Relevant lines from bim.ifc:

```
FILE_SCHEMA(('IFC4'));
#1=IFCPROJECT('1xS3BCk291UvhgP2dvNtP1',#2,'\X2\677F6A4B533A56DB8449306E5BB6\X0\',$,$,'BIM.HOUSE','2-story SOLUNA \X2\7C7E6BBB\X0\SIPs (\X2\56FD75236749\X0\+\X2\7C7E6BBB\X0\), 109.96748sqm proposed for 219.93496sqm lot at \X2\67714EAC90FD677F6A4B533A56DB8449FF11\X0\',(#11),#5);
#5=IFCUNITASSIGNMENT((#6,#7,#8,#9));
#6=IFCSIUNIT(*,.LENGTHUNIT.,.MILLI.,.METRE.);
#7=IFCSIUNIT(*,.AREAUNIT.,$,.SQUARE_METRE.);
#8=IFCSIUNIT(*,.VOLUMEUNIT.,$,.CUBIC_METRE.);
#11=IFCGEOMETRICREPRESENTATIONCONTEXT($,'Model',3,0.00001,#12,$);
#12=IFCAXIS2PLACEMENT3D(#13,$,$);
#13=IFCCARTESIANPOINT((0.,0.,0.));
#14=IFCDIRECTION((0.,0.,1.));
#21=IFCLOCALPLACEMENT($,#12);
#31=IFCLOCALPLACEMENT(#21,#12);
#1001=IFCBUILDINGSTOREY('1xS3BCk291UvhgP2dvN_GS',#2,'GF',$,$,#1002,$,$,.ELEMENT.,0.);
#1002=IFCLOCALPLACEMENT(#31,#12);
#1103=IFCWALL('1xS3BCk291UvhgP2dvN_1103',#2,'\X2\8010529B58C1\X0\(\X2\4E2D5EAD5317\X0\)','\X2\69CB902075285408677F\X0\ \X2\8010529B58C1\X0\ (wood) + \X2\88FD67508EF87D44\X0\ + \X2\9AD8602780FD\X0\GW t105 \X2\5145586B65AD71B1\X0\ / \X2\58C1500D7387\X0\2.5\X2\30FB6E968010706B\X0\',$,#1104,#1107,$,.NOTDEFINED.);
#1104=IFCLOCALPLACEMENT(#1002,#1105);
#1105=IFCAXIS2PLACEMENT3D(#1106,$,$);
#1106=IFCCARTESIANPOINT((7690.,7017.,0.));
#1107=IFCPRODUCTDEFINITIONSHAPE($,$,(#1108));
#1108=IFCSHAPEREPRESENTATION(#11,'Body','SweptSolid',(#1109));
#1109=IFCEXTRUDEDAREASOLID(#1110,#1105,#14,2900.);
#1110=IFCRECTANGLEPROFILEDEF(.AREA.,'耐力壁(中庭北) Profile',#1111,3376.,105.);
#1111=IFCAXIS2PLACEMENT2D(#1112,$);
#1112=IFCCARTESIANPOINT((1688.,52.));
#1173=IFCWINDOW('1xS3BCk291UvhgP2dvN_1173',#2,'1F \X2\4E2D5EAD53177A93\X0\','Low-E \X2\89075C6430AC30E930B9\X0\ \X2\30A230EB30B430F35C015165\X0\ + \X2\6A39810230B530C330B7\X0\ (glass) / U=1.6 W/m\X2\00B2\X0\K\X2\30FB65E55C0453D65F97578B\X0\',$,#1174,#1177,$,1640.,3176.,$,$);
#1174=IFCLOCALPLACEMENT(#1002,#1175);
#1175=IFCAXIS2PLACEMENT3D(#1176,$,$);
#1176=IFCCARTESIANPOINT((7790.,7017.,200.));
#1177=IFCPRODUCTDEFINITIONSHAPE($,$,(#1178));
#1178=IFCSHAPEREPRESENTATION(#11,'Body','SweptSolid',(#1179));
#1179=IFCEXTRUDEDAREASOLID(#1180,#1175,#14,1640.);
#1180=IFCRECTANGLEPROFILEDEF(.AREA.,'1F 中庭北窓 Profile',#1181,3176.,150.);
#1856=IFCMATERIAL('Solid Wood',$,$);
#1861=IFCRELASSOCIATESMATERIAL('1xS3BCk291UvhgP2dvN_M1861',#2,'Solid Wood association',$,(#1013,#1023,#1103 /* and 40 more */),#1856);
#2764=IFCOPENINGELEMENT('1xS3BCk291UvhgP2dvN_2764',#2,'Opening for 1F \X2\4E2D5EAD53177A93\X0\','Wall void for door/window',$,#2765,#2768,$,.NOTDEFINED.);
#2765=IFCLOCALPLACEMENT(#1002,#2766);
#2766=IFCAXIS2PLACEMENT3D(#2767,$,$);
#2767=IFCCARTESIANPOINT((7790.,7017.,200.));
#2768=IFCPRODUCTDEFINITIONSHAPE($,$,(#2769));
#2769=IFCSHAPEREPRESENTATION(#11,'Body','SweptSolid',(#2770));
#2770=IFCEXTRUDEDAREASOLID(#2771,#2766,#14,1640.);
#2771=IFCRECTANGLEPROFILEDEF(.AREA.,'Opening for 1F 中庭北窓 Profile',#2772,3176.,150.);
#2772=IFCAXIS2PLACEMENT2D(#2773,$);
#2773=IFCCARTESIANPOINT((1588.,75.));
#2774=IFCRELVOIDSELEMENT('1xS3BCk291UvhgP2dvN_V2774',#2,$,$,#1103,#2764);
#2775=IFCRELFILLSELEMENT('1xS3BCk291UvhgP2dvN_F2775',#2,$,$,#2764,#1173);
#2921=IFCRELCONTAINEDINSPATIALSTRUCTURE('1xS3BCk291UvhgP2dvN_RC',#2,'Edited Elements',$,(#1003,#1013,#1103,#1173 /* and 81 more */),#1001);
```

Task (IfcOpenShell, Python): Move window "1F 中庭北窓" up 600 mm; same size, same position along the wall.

```python
import numpy as np
import ifcopenshell
import ifcopenshell.api.geometry
import ifcopenshell.util.placement
import ifcopenshell.util.unit

model = ifcopenshell.open("bim.ifc")
unit_scale = ifcopenshell.util.unit.calculate_unit_scale(model)

window = model.by_guid("1xS3BCk291UvhgP2dvN_1173")
opening = window.FillsVoids[0].RelatingOpeningElement
dz = 0.6 / unit_scale

shift = np.array([0.0, 0.0, dz])
# The window is not placed relative to its opening, so move both.
for product in (opening, window):
    matrix = ifcopenshell.util.placement.get_local_placement(product.ObjectPlacement)
    matrix[:3, 3] += shift
    ifcopenshell.api.geometry.edit_object_placement(model, product=product, matrix=matrix, is_si=False)

print(f"moved by {dz * unit_scale:+.3f} m")

model.write("bim_v2.ifc")
```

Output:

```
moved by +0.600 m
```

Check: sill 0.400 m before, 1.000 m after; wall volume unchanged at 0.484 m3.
